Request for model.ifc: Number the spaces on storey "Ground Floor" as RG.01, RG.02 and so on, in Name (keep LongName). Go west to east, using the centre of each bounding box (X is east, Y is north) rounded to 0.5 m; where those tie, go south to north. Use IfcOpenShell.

First a look at what the model holds.

```python
import ifcopenshell
import ifcopenshell.util.element
import ifcopenshell.util.placement

model = ifcopenshell.open("model.ifc")
print(model.schema)
storey = next(s for s in model.by_type("IfcBuildingStorey") if s.Name == "Ground Floor")
spaces = [e for e in ifcopenshell.util.element.get_decomposition(storey) if e.is_a("IfcSpace")]
for e in sorted(spaces, key=lambda e: e.id()):
    origin = ifcopenshell.util.placement.get_local_placement(e.ObjectPlacement)[:3, 3]
    print(e.id(), e.Name, e.LongName, origin.round(2) + 0.0, sep=" | ")
```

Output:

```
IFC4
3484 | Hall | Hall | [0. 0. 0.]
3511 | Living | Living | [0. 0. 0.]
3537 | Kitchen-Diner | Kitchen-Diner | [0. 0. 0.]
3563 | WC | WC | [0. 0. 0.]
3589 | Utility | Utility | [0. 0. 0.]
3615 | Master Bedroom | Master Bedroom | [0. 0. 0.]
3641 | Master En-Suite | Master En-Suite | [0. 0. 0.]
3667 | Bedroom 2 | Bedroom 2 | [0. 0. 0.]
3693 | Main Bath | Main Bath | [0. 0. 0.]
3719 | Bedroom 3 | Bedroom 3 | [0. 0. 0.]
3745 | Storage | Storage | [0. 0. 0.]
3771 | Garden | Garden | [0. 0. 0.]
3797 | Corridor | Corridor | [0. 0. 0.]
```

```python
import ifcopenshell
import ifcopenshell.geom
import ifcopenshell.util.element
import ifcopenshell.util.shape

model = ifcopenshell.open("model.ifc")
settings = ifcopenshell.geom.settings()
settings.set("use-world-coords", True)


def centre(element):
    shape = ifcopenshell.geom.create_shape(settings, element)
    return ifcopenshell.util.shape.get_bbox_centroid(shape.geometry)


storey = next(s for s in model.by_type("IfcBuildingStorey") if s.Name == "Ground Floor")
spaces = [e for e in ifcopenshell.util.element.get_decomposition(storey) if e.is_a("IfcSpace")]

# Insertion points can sit at a corner or the storey origin, so sort by the geometry (in metres).
centres = {e: centre(e) for e in spaces}
spaces.sort(key=lambda e: (round(centres[e][0] / 0.5), centres[e][1]))

for i, e in enumerate(spaces, start=1):
    number = f"RG.{i:02d}"
    e.Name = number
    print(e.id(), number)

model.write("model_rev.ifc")
```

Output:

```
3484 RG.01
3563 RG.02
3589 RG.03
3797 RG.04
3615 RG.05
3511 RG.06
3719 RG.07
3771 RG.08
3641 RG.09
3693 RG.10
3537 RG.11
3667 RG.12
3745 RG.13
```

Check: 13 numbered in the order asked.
